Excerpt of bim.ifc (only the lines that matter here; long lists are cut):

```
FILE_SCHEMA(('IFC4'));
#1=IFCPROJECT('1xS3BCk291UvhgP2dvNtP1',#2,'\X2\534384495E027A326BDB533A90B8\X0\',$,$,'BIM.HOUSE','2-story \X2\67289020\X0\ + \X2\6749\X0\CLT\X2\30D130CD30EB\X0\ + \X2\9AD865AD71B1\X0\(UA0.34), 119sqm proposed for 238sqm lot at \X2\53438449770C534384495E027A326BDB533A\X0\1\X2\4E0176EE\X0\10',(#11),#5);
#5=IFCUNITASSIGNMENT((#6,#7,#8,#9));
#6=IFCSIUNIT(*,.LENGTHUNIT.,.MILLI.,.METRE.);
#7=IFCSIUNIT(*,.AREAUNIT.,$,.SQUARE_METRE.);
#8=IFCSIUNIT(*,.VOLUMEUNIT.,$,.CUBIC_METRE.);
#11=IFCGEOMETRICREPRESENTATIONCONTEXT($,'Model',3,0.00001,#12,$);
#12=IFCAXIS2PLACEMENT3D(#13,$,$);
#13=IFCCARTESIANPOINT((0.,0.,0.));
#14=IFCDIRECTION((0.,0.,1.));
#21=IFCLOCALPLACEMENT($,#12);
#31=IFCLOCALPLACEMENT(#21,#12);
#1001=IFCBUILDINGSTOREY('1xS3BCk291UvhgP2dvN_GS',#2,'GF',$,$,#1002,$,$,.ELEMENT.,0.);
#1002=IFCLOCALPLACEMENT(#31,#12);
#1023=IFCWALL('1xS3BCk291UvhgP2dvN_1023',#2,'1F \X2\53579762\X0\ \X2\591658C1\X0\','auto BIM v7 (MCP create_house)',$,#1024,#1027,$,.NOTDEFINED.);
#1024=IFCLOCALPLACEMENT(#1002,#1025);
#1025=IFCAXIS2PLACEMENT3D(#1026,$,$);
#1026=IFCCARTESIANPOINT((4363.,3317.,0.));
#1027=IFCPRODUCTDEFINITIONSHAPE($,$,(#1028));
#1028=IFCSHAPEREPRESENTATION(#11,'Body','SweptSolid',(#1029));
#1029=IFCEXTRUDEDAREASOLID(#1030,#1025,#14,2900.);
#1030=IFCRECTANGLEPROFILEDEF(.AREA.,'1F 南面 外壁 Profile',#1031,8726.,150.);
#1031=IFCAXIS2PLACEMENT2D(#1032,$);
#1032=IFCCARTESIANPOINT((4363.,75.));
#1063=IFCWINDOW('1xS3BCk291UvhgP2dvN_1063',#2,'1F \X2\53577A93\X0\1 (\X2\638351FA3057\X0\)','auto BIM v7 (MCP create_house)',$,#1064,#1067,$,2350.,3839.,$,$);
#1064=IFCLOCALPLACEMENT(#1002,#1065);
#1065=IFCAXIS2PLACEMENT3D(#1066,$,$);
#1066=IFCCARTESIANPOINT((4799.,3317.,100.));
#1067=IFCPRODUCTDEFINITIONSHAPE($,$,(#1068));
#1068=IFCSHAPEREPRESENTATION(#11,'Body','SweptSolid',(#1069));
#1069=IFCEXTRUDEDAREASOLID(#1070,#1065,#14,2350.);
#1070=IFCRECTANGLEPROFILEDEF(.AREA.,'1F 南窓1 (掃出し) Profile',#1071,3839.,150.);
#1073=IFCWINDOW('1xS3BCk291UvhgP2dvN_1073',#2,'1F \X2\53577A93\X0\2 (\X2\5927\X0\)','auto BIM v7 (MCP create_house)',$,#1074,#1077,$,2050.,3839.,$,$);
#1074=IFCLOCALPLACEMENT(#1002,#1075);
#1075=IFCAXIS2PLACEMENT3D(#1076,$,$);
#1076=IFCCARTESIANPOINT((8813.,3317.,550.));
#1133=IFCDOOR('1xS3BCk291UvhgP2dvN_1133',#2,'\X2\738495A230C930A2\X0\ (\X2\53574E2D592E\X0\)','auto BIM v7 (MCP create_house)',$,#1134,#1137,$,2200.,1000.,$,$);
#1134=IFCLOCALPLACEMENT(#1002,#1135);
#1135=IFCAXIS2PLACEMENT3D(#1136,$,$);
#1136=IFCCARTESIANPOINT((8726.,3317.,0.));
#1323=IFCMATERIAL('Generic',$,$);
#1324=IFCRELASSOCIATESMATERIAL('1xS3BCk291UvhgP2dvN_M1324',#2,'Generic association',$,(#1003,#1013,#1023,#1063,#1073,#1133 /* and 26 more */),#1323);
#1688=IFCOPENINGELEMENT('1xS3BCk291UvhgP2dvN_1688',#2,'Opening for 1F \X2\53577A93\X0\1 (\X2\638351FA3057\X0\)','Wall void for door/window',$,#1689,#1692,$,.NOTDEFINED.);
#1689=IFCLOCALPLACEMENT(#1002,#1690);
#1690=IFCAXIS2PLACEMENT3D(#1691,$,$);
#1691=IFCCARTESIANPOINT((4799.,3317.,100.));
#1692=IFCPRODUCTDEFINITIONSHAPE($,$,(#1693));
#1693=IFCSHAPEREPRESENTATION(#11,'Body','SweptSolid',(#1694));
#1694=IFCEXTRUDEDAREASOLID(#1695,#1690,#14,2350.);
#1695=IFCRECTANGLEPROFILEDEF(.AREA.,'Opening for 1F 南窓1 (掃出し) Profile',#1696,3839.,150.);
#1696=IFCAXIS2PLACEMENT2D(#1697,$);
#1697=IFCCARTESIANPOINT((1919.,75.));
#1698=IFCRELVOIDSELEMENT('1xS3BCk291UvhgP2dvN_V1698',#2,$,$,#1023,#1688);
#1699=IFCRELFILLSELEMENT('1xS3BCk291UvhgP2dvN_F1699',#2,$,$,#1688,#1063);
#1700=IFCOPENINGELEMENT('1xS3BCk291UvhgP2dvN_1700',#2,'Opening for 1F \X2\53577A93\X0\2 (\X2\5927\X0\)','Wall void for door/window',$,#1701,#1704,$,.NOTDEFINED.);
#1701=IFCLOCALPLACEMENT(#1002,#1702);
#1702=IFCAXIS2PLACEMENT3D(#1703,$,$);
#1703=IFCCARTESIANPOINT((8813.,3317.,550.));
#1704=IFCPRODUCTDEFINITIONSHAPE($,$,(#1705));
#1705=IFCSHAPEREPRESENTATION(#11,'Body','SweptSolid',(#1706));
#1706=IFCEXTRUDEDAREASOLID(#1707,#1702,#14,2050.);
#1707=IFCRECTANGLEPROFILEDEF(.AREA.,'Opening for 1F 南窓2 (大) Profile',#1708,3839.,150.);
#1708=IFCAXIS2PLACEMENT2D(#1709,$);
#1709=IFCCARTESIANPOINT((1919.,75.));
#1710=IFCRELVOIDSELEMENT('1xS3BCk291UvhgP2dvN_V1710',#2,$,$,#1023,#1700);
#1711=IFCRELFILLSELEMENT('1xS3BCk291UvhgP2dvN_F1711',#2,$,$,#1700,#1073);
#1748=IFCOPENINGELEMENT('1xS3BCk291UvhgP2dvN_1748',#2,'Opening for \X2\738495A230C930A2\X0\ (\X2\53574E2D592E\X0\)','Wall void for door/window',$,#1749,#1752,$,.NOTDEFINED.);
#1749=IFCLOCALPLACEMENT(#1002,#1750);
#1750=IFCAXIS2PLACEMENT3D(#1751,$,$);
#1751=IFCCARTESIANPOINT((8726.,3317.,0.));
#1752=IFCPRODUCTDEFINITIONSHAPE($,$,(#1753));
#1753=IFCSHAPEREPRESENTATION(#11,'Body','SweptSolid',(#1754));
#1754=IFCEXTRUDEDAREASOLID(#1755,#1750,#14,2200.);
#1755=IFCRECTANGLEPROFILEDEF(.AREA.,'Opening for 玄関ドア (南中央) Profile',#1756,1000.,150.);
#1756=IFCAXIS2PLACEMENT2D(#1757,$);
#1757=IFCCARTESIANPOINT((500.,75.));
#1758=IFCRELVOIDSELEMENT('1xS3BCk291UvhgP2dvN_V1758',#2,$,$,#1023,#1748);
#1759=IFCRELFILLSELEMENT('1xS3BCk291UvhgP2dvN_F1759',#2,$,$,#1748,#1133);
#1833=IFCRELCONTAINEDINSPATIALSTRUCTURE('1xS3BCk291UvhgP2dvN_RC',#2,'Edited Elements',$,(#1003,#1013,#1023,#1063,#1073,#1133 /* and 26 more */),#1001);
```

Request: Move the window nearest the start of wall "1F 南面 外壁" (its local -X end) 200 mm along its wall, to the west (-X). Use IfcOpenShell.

```python
import ifcopenshell
import ifcopenshell.api.geometry
import ifcopenshell.util.placement
import ifcopenshell.util.unit

model = ifcopenshell.open("bim.ifc")
unit_scale = ifcopenshell.util.unit.calculate_unit_scale(model)

window = model.by_guid("1xS3BCk291UvhgP2dvN_1063")
opening = window.FillsVoids[0].RelatingOpeningElement
wall = opening.VoidsElements[0].RelatingBuildingElement

wall_matrix = ifcopenshell.util.placement.get_local_placement(wall.ObjectPlacement)
shift = wall_matrix[:3, 0] * -0.2 / unit_scale
before = ifcopenshell.util.placement.get_local_placement(window.ObjectPlacement)[:3, 3].copy()

# The window is not placed relative to its opening, so move both.
for product in (opening, window):
    matrix = ifcopenshell.util.placement.get_local_placement(product.ObjectPlacement)
    matrix[:3, 3] += shift
    ifcopenshell.api.geometry.edit_object_placement(model, product=product, matrix=matrix, is_si=False)

after = ifcopenshell.util.placement.get_local_placement(window.ObjectPlacement)[:3, 3]
print("window moved by", (after - before).round(3) + 0.0)

model.write("bim-out.ifc")
```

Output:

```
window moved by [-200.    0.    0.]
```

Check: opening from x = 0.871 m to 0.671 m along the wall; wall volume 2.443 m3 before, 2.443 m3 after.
